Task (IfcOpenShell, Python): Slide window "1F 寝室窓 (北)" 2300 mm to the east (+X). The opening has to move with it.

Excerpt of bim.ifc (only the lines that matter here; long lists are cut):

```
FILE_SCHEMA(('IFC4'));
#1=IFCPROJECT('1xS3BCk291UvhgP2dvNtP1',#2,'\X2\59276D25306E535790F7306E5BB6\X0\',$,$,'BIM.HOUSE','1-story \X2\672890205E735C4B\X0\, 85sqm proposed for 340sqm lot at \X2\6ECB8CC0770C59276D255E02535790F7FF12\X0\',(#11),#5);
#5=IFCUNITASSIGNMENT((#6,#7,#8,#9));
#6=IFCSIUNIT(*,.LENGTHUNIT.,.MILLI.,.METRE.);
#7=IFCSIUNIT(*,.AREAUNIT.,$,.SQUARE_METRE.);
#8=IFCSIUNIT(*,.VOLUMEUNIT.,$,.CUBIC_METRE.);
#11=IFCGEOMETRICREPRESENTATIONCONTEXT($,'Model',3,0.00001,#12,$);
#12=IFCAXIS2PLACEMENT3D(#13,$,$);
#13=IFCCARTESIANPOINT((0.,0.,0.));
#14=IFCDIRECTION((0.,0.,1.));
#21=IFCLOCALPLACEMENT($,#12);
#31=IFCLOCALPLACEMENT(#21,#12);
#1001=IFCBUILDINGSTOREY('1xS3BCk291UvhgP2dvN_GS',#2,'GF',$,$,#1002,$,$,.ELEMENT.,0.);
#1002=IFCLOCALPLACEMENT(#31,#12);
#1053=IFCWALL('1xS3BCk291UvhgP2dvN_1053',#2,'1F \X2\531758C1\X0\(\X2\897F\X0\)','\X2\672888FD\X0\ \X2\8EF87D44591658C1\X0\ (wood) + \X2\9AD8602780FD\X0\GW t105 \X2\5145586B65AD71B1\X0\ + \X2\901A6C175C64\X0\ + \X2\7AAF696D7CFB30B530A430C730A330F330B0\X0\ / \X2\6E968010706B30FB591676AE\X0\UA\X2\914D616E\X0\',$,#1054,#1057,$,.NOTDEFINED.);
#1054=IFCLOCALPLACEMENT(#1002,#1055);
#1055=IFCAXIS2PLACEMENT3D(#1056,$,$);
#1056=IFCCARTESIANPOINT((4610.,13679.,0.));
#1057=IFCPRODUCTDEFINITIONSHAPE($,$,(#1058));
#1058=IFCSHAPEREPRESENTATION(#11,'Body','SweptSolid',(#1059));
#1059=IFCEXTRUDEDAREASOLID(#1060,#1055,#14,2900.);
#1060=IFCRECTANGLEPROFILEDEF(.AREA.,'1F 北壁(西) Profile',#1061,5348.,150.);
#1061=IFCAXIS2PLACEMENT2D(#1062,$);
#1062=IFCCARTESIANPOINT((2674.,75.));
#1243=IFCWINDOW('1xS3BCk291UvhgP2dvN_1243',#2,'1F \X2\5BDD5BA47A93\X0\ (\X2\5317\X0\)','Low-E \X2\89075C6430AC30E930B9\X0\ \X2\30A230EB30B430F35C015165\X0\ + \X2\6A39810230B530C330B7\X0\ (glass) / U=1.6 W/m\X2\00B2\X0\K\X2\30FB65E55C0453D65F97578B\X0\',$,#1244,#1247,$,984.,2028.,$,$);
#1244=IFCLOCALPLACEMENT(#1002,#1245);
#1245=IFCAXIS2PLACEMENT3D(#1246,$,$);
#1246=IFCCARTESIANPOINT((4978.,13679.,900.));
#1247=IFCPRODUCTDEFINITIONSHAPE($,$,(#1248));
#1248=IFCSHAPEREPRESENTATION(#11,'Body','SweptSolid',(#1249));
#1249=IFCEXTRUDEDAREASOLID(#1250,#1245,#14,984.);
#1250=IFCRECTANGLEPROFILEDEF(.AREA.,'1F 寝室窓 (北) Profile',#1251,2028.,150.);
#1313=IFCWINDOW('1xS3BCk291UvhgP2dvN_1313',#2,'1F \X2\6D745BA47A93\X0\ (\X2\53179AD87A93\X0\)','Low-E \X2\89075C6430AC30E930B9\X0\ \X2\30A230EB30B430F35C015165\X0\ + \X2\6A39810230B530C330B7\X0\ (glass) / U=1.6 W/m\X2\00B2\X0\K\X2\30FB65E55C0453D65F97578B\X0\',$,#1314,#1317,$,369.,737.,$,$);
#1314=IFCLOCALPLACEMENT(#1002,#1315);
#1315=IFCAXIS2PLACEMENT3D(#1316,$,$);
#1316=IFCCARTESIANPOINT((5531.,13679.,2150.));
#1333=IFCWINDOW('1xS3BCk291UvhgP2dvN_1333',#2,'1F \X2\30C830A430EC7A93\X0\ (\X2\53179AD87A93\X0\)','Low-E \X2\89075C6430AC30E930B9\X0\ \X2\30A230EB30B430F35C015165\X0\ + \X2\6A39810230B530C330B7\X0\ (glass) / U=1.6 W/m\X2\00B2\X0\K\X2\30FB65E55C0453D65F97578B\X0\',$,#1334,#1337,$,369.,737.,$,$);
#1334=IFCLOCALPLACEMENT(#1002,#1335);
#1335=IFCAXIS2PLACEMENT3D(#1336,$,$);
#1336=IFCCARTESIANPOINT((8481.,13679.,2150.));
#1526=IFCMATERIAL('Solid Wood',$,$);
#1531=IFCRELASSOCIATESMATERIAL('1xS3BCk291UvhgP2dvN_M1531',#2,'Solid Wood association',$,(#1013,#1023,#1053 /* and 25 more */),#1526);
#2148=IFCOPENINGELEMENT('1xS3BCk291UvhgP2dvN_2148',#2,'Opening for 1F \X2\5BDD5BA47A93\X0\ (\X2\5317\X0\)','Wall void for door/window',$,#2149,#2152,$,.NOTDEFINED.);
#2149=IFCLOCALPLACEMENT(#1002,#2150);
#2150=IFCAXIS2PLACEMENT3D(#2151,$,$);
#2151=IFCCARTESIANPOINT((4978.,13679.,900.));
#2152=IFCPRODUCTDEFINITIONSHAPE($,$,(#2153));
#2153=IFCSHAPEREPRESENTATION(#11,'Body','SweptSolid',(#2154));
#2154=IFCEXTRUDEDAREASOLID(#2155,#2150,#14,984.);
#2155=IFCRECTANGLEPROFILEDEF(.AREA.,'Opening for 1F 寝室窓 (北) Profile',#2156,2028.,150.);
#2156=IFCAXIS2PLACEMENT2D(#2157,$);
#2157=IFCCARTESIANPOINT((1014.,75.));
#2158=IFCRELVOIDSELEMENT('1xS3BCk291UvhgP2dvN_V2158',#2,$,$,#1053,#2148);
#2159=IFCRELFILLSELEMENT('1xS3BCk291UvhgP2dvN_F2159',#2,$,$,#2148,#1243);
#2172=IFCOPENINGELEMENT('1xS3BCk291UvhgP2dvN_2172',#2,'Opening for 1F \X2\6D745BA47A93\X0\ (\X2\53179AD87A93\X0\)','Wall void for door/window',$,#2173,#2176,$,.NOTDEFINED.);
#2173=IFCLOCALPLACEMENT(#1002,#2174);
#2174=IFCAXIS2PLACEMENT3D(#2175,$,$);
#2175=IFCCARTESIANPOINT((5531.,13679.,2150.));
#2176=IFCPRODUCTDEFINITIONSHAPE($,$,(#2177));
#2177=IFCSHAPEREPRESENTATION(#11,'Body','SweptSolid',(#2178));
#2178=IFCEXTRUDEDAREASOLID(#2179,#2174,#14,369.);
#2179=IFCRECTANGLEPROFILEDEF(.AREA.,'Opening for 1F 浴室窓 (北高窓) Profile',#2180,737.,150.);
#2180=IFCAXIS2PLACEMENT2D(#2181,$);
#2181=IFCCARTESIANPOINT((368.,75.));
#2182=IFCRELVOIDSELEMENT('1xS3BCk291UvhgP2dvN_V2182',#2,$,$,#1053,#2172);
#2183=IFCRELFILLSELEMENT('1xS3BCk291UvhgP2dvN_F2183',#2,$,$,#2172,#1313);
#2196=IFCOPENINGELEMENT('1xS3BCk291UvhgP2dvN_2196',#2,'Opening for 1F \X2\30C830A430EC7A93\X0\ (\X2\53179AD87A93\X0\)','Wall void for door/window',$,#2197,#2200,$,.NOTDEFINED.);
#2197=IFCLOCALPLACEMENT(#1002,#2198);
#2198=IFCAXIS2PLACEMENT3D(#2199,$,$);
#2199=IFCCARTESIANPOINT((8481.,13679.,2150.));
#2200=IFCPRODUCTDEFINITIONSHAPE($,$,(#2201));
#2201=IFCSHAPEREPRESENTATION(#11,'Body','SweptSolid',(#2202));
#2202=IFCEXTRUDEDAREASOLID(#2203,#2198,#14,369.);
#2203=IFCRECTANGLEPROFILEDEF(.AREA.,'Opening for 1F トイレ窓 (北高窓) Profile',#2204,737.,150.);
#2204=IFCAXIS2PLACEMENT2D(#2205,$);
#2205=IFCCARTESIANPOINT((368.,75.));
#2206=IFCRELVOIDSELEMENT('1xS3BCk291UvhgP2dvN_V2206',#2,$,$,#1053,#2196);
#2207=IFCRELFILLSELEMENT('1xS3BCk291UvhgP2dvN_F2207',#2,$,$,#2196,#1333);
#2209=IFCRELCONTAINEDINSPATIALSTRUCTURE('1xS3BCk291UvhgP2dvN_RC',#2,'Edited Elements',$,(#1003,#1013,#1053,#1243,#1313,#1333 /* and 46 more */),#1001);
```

```python
import ifcopenshell
import ifcopenshell.api.geometry
import ifcopenshell.util.placement
import ifcopenshell.util.unit

model = ifcopenshell.open("bim.ifc")
unit_scale = ifcopenshell.util.unit.calculate_unit_scale(model)

window = model.by_guid("1xS3BCk291UvhgP2dvN_1243")
opening = window.FillsVoids[0].RelatingOpeningElement
wall = opening.VoidsElements[0].RelatingBuildingElement

wall_matrix = ifcopenshell.util.placement.get_local_placement(wall.ObjectPlacement)
shift = wall_matrix[:3, 0] * 2.3 / unit_scale
before = ifcopenshell.util.placement.get_local_placement(window.ObjectPlacement)[:3, 3].copy()

# The window is not placed relative to its opening, so move both.
for product in (opening, window):
    matrix = ifcopenshell.util.placement.get_local_placement(product.ObjectPlacement)
    matrix[:3, 3] += shift
    ifcopenshell.api.geometry.edit_object_placement(model, product=product, matrix=matrix, is_si=False)

after = ifcopenshell.util.placement.get_local_placement(window.ObjectPlacement)[:3, 3]
print("window moved by", (after - before).round(3) + 0.0)

model.write("bim_rev.ifc")
```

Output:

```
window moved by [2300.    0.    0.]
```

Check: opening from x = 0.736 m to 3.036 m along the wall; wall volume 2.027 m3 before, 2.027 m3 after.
